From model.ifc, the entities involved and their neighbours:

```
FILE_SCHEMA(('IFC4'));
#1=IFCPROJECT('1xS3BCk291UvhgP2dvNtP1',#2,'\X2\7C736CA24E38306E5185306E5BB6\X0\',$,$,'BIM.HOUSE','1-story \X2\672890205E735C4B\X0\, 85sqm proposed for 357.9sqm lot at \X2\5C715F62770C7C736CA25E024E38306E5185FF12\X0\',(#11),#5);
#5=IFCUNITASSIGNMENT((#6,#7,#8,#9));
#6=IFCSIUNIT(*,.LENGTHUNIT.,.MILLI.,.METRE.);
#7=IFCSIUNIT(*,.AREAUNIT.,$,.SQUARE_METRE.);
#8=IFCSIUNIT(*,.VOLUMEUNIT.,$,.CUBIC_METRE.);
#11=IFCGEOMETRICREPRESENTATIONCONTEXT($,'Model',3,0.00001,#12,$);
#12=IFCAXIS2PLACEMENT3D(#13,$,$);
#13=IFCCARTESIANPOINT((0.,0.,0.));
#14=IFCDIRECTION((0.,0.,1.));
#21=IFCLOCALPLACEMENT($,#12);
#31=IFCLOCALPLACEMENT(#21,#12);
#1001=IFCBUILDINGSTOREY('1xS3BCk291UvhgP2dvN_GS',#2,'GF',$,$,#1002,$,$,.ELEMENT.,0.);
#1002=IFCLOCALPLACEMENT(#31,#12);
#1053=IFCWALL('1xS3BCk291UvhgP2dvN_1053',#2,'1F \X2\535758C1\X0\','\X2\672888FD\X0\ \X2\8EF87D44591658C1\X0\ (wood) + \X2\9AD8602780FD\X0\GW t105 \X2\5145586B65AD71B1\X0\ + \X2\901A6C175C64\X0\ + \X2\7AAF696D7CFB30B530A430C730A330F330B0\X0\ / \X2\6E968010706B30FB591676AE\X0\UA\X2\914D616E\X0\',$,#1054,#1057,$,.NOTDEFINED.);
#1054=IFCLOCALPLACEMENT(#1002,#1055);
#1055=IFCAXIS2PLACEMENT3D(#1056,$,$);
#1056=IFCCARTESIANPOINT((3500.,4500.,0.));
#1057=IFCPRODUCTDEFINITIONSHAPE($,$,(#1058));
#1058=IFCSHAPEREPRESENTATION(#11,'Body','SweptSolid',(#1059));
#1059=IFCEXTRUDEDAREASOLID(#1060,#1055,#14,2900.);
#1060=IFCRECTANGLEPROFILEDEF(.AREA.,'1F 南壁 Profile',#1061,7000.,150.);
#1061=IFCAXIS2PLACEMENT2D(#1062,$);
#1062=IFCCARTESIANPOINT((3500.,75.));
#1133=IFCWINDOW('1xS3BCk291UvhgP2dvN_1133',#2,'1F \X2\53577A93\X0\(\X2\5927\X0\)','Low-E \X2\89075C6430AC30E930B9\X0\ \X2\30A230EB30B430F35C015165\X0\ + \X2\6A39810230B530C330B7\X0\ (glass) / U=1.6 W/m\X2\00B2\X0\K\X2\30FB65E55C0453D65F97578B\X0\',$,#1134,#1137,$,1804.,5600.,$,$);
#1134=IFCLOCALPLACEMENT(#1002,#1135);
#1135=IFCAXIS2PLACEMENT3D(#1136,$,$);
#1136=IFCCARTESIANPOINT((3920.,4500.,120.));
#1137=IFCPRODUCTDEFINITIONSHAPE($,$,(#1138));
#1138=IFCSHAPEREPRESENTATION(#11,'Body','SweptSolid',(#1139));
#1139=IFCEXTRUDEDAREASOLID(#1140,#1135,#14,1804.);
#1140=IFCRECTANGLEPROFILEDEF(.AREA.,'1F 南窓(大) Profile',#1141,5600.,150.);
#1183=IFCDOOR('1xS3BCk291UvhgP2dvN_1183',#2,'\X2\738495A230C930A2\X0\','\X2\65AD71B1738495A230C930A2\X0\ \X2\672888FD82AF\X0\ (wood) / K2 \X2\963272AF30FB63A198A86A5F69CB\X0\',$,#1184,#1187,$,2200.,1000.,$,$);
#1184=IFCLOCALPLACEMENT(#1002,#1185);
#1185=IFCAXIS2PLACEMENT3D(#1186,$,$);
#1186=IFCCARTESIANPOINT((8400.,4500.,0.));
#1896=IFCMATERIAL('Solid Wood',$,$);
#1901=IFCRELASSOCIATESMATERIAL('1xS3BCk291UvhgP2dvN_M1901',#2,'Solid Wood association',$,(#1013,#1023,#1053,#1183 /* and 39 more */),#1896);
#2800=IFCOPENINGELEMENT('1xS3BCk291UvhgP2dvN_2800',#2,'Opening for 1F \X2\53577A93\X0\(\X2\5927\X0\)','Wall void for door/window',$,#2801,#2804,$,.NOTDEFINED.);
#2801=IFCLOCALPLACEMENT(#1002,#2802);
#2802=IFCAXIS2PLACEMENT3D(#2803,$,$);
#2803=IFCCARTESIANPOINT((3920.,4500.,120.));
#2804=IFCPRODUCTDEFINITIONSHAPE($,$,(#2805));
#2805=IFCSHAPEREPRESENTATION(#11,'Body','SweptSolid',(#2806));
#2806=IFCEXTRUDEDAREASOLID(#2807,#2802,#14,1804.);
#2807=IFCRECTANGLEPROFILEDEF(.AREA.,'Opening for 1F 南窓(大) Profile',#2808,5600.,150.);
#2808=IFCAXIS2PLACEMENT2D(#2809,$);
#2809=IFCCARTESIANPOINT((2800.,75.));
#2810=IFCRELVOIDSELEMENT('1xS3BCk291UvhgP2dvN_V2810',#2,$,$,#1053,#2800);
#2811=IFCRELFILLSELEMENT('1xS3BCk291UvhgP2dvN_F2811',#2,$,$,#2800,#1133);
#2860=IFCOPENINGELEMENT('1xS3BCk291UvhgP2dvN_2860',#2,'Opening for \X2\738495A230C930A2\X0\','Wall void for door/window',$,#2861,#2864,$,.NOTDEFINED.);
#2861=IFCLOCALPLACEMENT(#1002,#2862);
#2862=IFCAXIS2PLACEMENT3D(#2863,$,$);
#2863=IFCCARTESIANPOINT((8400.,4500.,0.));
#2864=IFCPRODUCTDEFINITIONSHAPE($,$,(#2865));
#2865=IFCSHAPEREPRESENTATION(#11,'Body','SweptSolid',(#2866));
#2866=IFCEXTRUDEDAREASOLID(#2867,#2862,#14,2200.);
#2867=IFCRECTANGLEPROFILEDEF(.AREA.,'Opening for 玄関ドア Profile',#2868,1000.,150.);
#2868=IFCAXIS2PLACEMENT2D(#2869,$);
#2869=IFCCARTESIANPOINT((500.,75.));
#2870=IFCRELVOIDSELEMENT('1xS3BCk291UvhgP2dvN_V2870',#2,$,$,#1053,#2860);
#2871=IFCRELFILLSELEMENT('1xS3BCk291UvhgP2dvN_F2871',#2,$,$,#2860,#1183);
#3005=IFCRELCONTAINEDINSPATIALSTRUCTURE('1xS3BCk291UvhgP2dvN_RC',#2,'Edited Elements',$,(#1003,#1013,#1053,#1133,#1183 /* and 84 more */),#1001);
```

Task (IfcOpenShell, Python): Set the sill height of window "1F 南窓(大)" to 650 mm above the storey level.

```python
import numpy as np
import ifcopenshell
import ifcopenshell.api.geometry
import ifcopenshell.geom
import ifcopenshell.util.element
import ifcopenshell.util.placement
import ifcopenshell.util.shape
import ifcopenshell.util.unit

model = ifcopenshell.open("model.ifc")
unit_scale = ifcopenshell.util.unit.calculate_unit_scale(model)

window = model.by_id(1133)
opening = window.FillsVoids[0].RelatingOpeningElement
storey = ifcopenshell.util.element.get_container(window, ifc_class="IfcBuildingStorey")
level = ifcopenshell.util.placement.get_local_placement(storey.ObjectPlacement)[2, 3]

# The opening's origin need not be at the sill, so measure its lowest point.
shape = ifcopenshell.geom.create_shape(ifcopenshell.geom.settings(), opening)
bottom = ifcopenshell.util.shape.get_shape_bottom_elevation(shape, shape.geometry) / unit_scale
dz = level + 650.0 - bottom

shift = np.array([0.0, 0.0, dz])
# The window is not placed relative to its opening, so move both.
for product in (opening, window):
    matrix = ifcopenshell.util.placement.get_local_placement(product.ObjectPlacement)
    matrix[:3, 3] += shift
    ifcopenshell.api.geometry.edit_object_placement(model, product=product, matrix=matrix, is_si=False)

print(f"moved by {dz * unit_scale:+.3f} m")

model.write("model_v2.ifc")
```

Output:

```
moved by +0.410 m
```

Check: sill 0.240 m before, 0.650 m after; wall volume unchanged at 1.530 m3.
